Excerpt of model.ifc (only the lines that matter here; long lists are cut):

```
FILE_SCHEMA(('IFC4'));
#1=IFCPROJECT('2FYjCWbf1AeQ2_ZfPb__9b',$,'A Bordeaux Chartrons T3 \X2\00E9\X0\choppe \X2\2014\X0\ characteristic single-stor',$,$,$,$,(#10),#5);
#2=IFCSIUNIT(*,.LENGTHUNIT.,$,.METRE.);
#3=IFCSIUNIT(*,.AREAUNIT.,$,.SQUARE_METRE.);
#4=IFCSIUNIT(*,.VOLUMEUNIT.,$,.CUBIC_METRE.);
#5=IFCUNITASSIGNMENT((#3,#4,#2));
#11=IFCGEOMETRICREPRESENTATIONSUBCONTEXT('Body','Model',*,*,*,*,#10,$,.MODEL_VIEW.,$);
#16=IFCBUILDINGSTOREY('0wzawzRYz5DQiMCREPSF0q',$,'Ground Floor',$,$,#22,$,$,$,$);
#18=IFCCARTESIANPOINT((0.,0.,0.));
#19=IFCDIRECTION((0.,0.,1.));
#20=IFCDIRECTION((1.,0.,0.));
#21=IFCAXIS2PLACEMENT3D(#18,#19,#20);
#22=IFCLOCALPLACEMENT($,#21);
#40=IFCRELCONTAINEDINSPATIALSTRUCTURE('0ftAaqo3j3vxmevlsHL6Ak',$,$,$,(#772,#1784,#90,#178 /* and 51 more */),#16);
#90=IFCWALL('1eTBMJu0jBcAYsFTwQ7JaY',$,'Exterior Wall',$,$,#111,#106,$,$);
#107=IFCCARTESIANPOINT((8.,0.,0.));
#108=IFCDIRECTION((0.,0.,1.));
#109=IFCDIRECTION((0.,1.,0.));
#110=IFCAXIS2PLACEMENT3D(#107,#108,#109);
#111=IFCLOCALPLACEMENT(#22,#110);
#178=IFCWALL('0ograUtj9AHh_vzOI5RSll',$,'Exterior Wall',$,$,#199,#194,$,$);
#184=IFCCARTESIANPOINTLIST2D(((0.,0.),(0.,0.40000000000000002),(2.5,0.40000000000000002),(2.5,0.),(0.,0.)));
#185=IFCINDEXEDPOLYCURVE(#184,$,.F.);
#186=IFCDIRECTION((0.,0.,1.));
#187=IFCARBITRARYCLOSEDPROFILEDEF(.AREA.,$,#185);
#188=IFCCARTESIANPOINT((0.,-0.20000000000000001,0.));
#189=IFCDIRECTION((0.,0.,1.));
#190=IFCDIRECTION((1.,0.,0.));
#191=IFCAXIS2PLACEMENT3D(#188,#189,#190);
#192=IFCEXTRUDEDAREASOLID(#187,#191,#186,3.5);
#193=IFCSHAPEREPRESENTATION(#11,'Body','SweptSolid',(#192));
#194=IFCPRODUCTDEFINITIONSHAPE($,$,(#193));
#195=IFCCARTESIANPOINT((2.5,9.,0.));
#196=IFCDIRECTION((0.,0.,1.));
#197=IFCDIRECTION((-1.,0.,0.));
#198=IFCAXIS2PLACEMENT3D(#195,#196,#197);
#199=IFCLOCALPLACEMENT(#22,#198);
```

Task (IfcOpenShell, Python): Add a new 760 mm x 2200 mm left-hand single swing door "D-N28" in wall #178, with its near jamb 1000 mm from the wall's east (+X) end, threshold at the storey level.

```python
import numpy as np
import ifcopenshell
import ifcopenshell.api.feature
import ifcopenshell.api.geometry
import ifcopenshell.api.root
import ifcopenshell.api.spatial
import ifcopenshell.geom
import ifcopenshell.util.element
import ifcopenshell.util.placement
import ifcopenshell.util.representation
import ifcopenshell.util.shape
import ifcopenshell.util.unit

model = ifcopenshell.open("model.ifc")
unit_scale = ifcopenshell.util.unit.calculate_unit_scale(model)
settings = ifcopenshell.geom.settings()


def volume(element):
    """Net volume in cubic metres, openings subtracted."""
    shape = ifcopenshell.geom.create_shape(settings, element)
    return ifcopenshell.util.shape.get_volume(shape.geometry)


wall = model.by_id(178)
storey = ifcopenshell.util.element.get_container(wall, ifc_class="IfcBuildingStorey")
context = ifcopenshell.util.representation.get_context(model, "Model", "Body", "MODEL_VIEW")
before = volume(wall)

width, height, from_end, sill = 0.76, 2.2, 1, 0.0  # metres

# The wall runs along its own X axis, and the end named is its -X end.
wall_shape = ifcopenshell.geom.create_shape(settings, wall)
x, y, z = ifcopenshell.util.shape.get_vertices(wall_shape.geometry).T
start = x.min() + from_end
face, thickness = float(y.min()), float(y.max() - y.min())
wall_matrix = ifcopenshell.util.placement.get_local_placement(wall.ObjectPlacement)
level = ifcopenshell.util.placement.get_local_placement(storey.ObjectPlacement)[2, 3]


def in_wall(x, y):
    """Placement at x, y metres in the wall's axes, at sill height."""
    matrix = wall_matrix.copy()
    matrix[:, 3] = wall_matrix @ np.array([x / unit_scale, y / unit_scale, 0.0, 1.0])
    matrix[2, 3] = level + sill / unit_scale
    return matrix


# Opening: a box that overshoots both wall faces by 50 mm.
opening = ifcopenshell.api.root.create_entity(model, ifc_class="IfcOpeningElement", predefined_type="OPENING")
box = ifcopenshell.api.geometry.add_wall_representation(
    model, context=context, length=width, height=height, thickness=thickness + 0.1
)
ifcopenshell.api.geometry.assign_representation(model, product=opening, representation=box)
ifcopenshell.api.geometry.edit_object_placement(model, product=opening, matrix=in_wall(start, face - 0.05), is_si=False)
ifcopenshell.api.feature.add_feature(model, feature=opening, element=wall)

door = ifcopenshell.api.root.create_entity(model, ifc_class="IfcDoor", name="D-N28", predefined_type="DOOR")
door.OverallWidth, door.OverallHeight = width / unit_scale, height / unit_scale
door.OperationType = "SINGLE_SWING_LEFT"
body = ifcopenshell.api.geometry.add_door_representation(
    model,
    context=context,
    overall_width=door.OverallWidth,
    overall_height=door.OverallHeight,
    operation_type="SINGLE_SWING_LEFT",
    lining_properties={"LiningDepth": thickness / unit_scale, "ThresholdDepth": thickness / unit_scale},
)
ifcopenshell.api.geometry.assign_representation(model, product=door, representation=body)
ifcopenshell.api.spatial.assign_container(model, products=[door], relating_structure=storey)
ifcopenshell.api.feature.add_filling(model, opening=opening, element=door)

# The lining spans the wall, so the door starts at the wall face.
ifcopenshell.api.geometry.edit_object_placement(model, product=door, matrix=in_wall(start, face), is_si=False)

after = volume(wall)

print(f"wall volume {before:.3f} -> {after:.3f} m3")

model.write("model_updated.ifc")
```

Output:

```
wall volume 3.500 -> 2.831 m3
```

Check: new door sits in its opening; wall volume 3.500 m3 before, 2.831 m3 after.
